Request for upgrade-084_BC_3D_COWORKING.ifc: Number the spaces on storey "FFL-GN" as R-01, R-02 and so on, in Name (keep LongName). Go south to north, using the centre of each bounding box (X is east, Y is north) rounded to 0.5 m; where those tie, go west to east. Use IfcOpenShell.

First a look at what the model holds.

```python
import ifcopenshell
import ifcopenshell.util.element
import ifcopenshell.util.placement

model = ifcopenshell.open("upgrade-084_BC_3D_COWORKING.ifc")
print(model.schema)
storey = next(s for s in model.by_type("IfcBuildingStorey") if s.Name == "FFL-GN")
spaces = [e for e in ifcopenshell.util.element.get_decomposition(storey) if e.is_a("IfcSpace")]
for e in sorted(spaces, key=lambda e: e.id()):
    origin = ifcopenshell.util.placement.get_local_placement(e.ObjectPlacement)[:3, 3]
    print(e.id(), e.Name, e.LongName, origin.round(2) + 0.0, sep=" | ")
```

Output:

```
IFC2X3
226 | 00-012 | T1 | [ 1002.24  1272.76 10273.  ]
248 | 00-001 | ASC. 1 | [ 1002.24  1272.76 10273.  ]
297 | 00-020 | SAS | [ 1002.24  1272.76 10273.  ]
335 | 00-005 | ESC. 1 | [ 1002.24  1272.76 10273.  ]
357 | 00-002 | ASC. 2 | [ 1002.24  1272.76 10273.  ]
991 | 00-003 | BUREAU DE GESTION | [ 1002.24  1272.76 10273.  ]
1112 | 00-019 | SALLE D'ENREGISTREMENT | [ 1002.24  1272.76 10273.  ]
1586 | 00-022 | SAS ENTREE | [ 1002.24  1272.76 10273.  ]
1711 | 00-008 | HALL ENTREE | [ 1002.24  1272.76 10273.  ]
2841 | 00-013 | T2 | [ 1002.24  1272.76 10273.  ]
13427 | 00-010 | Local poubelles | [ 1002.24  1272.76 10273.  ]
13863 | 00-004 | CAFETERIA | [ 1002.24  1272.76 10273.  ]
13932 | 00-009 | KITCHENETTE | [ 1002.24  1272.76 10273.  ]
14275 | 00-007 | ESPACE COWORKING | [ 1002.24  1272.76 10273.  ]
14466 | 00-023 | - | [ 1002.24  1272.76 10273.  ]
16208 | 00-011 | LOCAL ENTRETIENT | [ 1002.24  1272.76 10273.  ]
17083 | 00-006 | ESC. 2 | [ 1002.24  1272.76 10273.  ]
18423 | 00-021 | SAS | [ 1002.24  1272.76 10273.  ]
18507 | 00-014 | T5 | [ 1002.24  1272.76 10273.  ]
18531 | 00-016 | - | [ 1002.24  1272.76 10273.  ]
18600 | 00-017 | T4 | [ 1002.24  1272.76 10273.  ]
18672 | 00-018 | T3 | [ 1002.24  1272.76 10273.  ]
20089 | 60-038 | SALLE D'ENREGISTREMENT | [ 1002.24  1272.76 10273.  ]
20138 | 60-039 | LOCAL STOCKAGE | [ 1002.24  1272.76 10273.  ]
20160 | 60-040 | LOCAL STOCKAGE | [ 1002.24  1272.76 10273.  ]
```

```python
import ifcopenshell
import ifcopenshell.geom
import ifcopenshell.util.element
import ifcopenshell.util.shape

model = ifcopenshell.open("upgrade-084_BC_3D_COWORKING.ifc")
settings = ifcopenshell.geom.settings()
settings.set("use-world-coords", True)


def centre(element):
    shape = ifcopenshell.geom.create_shape(settings, element)
    return ifcopenshell.util.shape.get_bbox_centroid(shape.geometry)


storey = next(s for s in model.by_type("IfcBuildingStorey") if s.Name == "FFL-GN")
spaces = [e for e in ifcopenshell.util.element.get_decomposition(storey) if e.is_a("IfcSpace")]

# Insertion points can sit at a corner or the storey origin, so sort by the geometry (in metres).
centres = {e: centre(e) for e in spaces}
spaces.sort(key=lambda e: (round(centres[e][1] / 0.5), centres[e][0]))

for i, e in enumerate(spaces, start=1):
    number = f"R-{i:02d}"
    e.Name = number
    print(e.id(), number)

model.write("upgrade-084_BC_3D_COWORKING_updated.ifc")
```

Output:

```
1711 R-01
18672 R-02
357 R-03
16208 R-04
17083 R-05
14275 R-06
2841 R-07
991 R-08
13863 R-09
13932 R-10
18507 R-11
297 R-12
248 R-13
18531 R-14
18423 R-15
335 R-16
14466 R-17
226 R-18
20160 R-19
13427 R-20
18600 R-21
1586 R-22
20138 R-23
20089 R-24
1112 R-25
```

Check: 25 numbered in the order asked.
